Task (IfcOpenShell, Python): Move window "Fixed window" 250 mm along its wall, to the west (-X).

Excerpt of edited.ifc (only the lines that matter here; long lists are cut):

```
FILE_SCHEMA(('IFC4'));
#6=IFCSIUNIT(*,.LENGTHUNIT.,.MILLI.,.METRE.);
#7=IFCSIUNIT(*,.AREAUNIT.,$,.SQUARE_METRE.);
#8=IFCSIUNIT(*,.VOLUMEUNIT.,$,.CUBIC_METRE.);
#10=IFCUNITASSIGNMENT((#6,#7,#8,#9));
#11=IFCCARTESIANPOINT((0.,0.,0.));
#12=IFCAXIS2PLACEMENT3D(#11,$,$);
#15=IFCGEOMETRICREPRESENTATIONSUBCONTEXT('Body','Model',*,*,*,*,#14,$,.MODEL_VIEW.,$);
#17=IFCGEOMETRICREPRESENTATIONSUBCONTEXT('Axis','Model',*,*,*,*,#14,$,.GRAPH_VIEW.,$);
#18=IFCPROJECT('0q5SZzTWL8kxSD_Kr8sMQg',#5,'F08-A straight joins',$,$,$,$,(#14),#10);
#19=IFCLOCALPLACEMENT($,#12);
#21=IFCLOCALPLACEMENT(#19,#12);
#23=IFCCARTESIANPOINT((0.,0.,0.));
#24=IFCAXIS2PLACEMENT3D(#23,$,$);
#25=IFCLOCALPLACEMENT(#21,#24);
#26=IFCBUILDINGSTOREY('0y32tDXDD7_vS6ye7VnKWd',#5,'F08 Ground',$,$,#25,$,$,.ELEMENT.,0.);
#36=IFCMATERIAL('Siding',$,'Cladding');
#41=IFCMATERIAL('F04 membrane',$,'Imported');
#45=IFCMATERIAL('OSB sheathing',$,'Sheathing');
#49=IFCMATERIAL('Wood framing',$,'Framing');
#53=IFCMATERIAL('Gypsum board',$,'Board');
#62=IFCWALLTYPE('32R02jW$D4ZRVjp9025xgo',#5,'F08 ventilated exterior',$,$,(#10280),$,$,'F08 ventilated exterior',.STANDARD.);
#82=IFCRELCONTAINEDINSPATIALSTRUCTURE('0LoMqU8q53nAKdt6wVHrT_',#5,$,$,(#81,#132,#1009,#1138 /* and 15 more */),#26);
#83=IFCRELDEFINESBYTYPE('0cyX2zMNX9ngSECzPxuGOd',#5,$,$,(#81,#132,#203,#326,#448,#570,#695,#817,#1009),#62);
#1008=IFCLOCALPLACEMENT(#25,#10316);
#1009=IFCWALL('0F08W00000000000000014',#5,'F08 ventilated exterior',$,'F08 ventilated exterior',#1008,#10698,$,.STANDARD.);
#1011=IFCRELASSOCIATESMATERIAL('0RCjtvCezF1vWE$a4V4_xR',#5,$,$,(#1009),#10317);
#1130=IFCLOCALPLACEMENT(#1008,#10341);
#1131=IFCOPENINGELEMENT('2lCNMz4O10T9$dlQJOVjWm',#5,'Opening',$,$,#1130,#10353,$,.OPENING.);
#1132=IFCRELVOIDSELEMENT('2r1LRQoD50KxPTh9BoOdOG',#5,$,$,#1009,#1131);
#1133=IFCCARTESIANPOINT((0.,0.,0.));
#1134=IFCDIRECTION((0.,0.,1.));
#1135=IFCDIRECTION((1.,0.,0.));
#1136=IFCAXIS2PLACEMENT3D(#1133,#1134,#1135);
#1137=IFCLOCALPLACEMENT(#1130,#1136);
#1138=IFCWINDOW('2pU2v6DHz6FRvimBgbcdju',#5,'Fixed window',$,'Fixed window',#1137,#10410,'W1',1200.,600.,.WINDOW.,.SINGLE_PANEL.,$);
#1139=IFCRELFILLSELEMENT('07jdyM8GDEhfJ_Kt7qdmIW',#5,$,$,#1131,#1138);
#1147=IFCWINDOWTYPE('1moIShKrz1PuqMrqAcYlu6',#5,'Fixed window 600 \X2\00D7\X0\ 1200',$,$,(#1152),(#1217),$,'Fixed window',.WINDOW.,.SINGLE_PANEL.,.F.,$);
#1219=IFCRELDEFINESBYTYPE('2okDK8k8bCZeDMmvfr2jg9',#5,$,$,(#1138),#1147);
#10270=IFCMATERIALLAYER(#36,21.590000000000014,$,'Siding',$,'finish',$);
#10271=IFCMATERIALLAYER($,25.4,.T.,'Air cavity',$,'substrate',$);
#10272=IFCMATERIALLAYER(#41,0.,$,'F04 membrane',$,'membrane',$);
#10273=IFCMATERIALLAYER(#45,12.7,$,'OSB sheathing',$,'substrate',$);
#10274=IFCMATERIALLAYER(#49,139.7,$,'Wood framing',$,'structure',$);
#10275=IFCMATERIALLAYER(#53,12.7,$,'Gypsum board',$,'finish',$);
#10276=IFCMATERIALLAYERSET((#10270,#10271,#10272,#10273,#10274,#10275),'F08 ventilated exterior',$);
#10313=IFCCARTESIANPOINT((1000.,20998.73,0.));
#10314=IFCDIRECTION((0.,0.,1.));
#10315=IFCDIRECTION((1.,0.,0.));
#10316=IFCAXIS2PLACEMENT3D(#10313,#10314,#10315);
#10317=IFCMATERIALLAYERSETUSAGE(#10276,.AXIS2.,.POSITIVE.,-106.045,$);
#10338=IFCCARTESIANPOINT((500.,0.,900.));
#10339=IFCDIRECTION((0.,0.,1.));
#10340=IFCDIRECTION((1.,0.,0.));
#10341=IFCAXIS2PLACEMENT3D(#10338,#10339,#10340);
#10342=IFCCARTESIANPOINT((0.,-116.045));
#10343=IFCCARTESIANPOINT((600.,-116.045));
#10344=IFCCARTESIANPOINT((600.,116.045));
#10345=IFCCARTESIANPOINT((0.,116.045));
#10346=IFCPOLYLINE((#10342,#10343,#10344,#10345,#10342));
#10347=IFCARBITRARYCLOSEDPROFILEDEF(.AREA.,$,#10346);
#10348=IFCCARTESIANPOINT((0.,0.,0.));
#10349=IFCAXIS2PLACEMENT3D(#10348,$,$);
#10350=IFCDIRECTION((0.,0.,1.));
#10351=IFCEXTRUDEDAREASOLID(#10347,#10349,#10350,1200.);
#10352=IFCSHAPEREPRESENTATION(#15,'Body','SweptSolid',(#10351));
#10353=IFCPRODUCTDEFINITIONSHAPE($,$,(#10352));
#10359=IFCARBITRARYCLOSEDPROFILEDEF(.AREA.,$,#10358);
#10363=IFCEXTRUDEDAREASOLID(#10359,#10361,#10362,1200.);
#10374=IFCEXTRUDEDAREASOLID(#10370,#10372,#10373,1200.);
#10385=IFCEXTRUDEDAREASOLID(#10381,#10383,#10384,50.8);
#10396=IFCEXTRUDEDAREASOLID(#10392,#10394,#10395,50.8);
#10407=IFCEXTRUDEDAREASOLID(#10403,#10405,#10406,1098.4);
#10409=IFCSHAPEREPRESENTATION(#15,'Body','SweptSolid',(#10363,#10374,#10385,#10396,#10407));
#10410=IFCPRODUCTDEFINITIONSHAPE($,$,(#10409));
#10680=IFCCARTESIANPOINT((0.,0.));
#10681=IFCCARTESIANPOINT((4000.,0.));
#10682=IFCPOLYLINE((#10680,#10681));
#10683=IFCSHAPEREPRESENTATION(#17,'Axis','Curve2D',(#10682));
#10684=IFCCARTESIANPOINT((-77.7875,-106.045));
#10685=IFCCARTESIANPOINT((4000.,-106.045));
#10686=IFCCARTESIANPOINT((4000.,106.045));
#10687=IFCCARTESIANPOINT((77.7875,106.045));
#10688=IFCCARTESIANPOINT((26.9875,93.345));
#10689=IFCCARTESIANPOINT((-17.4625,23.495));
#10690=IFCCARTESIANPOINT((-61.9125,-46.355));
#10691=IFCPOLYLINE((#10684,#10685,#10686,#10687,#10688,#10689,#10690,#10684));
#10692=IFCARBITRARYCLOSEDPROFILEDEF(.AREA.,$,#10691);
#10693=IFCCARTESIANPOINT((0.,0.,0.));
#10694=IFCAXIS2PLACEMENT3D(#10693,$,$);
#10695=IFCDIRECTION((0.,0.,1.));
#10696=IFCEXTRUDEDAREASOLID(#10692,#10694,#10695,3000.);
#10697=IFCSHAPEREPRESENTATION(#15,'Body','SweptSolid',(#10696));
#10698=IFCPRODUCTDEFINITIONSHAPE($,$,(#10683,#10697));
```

```python
import ifcopenshell
import ifcopenshell.api.geometry
import ifcopenshell.util.placement

model = ifcopenshell.open("edited.ifc")

window = model.by_id(1138)
opening = window.FillsVoids[0].RelatingOpeningElement
wall = opening.VoidsElements[0].RelatingBuildingElement

wall_matrix = ifcopenshell.util.placement.get_local_placement(wall.ObjectPlacement)
shift = wall_matrix[:3, 0] * -250.0
before = ifcopenshell.util.placement.get_local_placement(window.ObjectPlacement)[:3, 3].copy()

# The window is placed relative to its opening, so it follows when the opening moves.
matrix = ifcopenshell.util.placement.get_local_placement(opening.ObjectPlacement)
matrix[:3, 3] += shift
ifcopenshell.api.geometry.edit_object_placement(
    model, product=opening, matrix=matrix, is_si=False, should_transform_children=True
)

after = ifcopenshell.util.placement.get_local_placement(window.ObjectPlacement)[:3, 3]
print("window moved by", (after - before).round(3) + 0.0)

model.write("edited-out.ifc")
```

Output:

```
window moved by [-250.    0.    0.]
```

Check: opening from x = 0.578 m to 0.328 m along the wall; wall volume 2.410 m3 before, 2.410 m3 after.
